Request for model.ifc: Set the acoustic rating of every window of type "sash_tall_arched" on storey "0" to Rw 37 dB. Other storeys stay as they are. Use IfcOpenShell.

First a look at what the model holds.

```python
import ifcopenshell
import ifcopenshell.util.element

model = ifcopenshell.open("model.ifc")
print(model.schema)
storey = next(s for s in model.by_type("IfcBuildingStorey") if s.Name == "0")
windows = [e for e in ifcopenshell.util.element.get_decomposition(storey) if e.is_a("IfcWindow")]
seen = {}
for e in windows:
    element_type = ifcopenshell.util.element.get_type(e)
    key = (element_type.Name if element_type != e and element_type else None, ifcopenshell.util.element.get_pset(e, "Pset_WindowCommon", "AcousticRating"))
    seen[key] = seen.get(key, 0) + 1
for (name, value), count in sorted(seen.items(), key=str):
    print(count, "x", name, "|", value)
```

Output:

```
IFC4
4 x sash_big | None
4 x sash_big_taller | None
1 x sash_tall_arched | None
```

```python
import ifcopenshell
import ifcopenshell.api.pset
import ifcopenshell.util.element

model = ifcopenshell.open("model.ifc")

storey = next(s for s in model.by_type("IfcBuildingStorey") if s.Name == "0")
windows = [e for e in ifcopenshell.util.element.get_decomposition(storey) if e.is_a("IfcWindow")]

count = 0
for e in windows:
    element_type = ifcopenshell.util.element.get_type(e)
    if element_type in (None, e) or element_type.Name != "sash_tall_arched":
        continue
    # add_pset returns the element's existing set when there is one.
    pset = ifcopenshell.api.pset.add_pset(model, product=e, name="Pset_WindowCommon")
    ifcopenshell.api.pset.edit_pset(model, pset=pset, properties={"AcousticRating": "Rw 37 dB"})
    count += 1

print(count, "windows updated")

model.write("model_edited.ifc")
```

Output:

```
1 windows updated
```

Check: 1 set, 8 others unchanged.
